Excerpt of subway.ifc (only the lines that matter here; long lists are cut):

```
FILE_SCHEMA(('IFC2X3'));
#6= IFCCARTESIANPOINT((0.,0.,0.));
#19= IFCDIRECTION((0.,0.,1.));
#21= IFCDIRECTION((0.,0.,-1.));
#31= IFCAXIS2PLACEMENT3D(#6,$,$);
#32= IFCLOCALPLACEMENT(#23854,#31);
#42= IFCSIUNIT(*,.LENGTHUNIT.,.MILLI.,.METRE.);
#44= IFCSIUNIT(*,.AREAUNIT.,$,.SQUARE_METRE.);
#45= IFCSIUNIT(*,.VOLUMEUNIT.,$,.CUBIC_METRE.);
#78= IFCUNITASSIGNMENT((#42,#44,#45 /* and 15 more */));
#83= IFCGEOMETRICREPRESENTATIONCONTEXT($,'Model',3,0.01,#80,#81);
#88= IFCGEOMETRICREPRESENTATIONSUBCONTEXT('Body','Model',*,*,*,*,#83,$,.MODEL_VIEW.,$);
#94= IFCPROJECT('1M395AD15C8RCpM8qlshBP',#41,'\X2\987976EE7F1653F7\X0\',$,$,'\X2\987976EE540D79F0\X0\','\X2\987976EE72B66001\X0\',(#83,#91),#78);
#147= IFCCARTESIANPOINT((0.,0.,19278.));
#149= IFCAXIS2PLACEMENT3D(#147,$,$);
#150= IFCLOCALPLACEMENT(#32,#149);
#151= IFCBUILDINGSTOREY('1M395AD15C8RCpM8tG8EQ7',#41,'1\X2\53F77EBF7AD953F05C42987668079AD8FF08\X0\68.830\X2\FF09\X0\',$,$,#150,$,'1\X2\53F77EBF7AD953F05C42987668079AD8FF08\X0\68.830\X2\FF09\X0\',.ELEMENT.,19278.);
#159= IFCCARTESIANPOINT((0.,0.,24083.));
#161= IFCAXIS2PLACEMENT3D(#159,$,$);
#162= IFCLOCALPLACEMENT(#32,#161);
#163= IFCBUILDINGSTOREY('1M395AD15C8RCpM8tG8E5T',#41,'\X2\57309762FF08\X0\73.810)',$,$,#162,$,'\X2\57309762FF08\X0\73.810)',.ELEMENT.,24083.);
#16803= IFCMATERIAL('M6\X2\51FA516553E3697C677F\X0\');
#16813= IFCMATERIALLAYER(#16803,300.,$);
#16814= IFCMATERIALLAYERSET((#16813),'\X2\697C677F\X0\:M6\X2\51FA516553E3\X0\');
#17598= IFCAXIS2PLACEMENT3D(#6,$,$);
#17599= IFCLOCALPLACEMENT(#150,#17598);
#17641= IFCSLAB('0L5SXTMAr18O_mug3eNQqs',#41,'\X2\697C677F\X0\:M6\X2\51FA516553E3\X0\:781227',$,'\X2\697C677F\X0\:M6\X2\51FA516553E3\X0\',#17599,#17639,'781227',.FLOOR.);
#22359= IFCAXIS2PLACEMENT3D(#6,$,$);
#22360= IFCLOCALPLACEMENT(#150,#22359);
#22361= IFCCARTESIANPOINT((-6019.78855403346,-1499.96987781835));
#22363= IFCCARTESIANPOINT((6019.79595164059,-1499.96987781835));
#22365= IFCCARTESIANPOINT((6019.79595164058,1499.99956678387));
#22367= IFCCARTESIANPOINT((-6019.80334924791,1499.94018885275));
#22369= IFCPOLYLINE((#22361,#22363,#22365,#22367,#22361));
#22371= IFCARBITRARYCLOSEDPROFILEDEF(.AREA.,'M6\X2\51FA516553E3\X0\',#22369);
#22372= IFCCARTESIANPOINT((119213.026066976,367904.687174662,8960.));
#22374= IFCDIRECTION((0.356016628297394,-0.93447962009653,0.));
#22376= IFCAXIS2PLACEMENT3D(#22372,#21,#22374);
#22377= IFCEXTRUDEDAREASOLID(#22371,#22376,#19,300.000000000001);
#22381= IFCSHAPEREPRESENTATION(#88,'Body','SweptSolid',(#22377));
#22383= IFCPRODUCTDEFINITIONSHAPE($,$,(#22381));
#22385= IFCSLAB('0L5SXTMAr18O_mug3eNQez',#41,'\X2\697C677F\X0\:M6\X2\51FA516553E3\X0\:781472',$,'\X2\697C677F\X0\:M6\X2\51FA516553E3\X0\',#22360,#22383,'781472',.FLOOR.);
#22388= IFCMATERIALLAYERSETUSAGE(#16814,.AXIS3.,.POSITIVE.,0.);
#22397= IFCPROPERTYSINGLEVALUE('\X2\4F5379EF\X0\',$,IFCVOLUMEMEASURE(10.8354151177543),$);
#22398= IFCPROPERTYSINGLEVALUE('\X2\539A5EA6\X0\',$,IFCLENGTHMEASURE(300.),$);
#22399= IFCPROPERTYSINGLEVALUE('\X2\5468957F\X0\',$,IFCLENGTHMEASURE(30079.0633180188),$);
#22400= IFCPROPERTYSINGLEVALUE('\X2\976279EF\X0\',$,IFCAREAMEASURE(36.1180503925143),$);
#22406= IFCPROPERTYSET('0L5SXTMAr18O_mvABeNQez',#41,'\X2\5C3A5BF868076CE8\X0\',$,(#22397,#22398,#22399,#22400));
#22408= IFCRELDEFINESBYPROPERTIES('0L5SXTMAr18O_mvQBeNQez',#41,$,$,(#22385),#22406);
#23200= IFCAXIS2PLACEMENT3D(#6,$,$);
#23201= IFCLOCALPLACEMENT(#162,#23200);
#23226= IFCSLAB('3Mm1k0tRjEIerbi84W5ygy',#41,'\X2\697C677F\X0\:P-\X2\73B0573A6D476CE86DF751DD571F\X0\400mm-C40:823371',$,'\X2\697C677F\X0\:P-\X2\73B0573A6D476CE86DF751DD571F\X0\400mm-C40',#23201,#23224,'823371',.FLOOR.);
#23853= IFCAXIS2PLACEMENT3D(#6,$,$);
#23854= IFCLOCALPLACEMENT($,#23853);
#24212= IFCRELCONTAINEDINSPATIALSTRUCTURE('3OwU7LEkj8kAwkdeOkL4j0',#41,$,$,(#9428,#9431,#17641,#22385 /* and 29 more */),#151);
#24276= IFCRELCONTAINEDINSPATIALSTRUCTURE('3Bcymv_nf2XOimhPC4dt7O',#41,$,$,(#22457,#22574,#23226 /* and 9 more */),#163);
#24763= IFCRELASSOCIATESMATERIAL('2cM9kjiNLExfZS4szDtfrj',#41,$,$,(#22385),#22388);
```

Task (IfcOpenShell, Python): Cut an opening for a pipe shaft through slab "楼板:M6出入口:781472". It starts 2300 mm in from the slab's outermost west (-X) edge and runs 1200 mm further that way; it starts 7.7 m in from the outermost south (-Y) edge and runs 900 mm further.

```python
import numpy as np
import ifcopenshell
import ifcopenshell.api.feature
import ifcopenshell.api.geometry
import ifcopenshell.api.pset
import ifcopenshell.api.root
import ifcopenshell.geom
import ifcopenshell.util.element
import ifcopenshell.util.placement
import ifcopenshell.util.representation
import ifcopenshell.util.shape
import ifcopenshell.util.unit

model = ifcopenshell.open("subway.ifc")
unit_scale = ifcopenshell.util.unit.calculate_unit_scale(model)
area_scale = ifcopenshell.util.unit.calculate_unit_scale(model, "AREAUNIT")
volume_scale = ifcopenshell.util.unit.calculate_unit_scale(model, "VOLUMEUNIT")
settings = ifcopenshell.geom.settings()


def volume(element):
    """Net volume in cubic metres, openings subtracted."""
    shape = ifcopenshell.geom.create_shape(settings, element)
    return ifcopenshell.util.shape.get_volume(shape.geometry)


slab = model.by_id(22385)
before = volume(slab)

# Extent in the slab's own axes, in metres. The edges named are its -X and -Y sides.
slab_shape = ifcopenshell.geom.create_shape(settings, slab)
vertices = ifcopenshell.util.shape.get_vertices(slab_shape.geometry)
x_min, y_min, bottom = vertices.min(axis=0)
top = vertices[:, 2].max()

opening = ifcopenshell.api.root.create_entity(model, ifc_class="IfcOpeningElement", name="Pipe shaft opening")
context = ifcopenshell.util.representation.get_context(model, "Model", "Body", "MODEL_VIEW")
width, depth = 1.2, 0.9
outline = [(0.0, 0.0), (width, 0.0), (width, depth), (0.0, depth), (0.0, 0.0)]
# Overshoot both faces by 50 mm so the cut is clean.
shape = ifcopenshell.api.geometry.add_slab_representation(
    model, context=context, depth=top - bottom + 0.1, polyline=outline
)
ifcopenshell.api.geometry.assign_representation(model, product=opening, representation=shape)

matrix = ifcopenshell.util.placement.get_local_placement(slab.ObjectPlacement)
matrix[:, 3] = matrix @ np.append(np.array([x_min + 2.3, y_min + 7.7, bottom - 0.05]) / unit_scale, 1.0)
ifcopenshell.api.geometry.edit_object_placement(model, product=opening, matrix=matrix, is_si=False)
ifcopenshell.api.feature.add_feature(model, feature=opening, element=slab)

after = volume(slab)

# Update the slab's stored quantities.
pset = model.by_id(ifcopenshell.util.element.get_pset(slab, "尺寸标注", should_inherit=False)["id"])
ifcopenshell.api.pset.edit_pset(model, pset=pset, properties={
    "体积": model.create_entity("IfcVolumeMeasure", after / volume_scale),
    "面积": model.create_entity("IfcAreaMeasure", after / (top - bottom) / area_scale),
})

print(f"slab volume {before:.3f} -> {after:.3f} m3")

model.write("subway_updated.ifc")
```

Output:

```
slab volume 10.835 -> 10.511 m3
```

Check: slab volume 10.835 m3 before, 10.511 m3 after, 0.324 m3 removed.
